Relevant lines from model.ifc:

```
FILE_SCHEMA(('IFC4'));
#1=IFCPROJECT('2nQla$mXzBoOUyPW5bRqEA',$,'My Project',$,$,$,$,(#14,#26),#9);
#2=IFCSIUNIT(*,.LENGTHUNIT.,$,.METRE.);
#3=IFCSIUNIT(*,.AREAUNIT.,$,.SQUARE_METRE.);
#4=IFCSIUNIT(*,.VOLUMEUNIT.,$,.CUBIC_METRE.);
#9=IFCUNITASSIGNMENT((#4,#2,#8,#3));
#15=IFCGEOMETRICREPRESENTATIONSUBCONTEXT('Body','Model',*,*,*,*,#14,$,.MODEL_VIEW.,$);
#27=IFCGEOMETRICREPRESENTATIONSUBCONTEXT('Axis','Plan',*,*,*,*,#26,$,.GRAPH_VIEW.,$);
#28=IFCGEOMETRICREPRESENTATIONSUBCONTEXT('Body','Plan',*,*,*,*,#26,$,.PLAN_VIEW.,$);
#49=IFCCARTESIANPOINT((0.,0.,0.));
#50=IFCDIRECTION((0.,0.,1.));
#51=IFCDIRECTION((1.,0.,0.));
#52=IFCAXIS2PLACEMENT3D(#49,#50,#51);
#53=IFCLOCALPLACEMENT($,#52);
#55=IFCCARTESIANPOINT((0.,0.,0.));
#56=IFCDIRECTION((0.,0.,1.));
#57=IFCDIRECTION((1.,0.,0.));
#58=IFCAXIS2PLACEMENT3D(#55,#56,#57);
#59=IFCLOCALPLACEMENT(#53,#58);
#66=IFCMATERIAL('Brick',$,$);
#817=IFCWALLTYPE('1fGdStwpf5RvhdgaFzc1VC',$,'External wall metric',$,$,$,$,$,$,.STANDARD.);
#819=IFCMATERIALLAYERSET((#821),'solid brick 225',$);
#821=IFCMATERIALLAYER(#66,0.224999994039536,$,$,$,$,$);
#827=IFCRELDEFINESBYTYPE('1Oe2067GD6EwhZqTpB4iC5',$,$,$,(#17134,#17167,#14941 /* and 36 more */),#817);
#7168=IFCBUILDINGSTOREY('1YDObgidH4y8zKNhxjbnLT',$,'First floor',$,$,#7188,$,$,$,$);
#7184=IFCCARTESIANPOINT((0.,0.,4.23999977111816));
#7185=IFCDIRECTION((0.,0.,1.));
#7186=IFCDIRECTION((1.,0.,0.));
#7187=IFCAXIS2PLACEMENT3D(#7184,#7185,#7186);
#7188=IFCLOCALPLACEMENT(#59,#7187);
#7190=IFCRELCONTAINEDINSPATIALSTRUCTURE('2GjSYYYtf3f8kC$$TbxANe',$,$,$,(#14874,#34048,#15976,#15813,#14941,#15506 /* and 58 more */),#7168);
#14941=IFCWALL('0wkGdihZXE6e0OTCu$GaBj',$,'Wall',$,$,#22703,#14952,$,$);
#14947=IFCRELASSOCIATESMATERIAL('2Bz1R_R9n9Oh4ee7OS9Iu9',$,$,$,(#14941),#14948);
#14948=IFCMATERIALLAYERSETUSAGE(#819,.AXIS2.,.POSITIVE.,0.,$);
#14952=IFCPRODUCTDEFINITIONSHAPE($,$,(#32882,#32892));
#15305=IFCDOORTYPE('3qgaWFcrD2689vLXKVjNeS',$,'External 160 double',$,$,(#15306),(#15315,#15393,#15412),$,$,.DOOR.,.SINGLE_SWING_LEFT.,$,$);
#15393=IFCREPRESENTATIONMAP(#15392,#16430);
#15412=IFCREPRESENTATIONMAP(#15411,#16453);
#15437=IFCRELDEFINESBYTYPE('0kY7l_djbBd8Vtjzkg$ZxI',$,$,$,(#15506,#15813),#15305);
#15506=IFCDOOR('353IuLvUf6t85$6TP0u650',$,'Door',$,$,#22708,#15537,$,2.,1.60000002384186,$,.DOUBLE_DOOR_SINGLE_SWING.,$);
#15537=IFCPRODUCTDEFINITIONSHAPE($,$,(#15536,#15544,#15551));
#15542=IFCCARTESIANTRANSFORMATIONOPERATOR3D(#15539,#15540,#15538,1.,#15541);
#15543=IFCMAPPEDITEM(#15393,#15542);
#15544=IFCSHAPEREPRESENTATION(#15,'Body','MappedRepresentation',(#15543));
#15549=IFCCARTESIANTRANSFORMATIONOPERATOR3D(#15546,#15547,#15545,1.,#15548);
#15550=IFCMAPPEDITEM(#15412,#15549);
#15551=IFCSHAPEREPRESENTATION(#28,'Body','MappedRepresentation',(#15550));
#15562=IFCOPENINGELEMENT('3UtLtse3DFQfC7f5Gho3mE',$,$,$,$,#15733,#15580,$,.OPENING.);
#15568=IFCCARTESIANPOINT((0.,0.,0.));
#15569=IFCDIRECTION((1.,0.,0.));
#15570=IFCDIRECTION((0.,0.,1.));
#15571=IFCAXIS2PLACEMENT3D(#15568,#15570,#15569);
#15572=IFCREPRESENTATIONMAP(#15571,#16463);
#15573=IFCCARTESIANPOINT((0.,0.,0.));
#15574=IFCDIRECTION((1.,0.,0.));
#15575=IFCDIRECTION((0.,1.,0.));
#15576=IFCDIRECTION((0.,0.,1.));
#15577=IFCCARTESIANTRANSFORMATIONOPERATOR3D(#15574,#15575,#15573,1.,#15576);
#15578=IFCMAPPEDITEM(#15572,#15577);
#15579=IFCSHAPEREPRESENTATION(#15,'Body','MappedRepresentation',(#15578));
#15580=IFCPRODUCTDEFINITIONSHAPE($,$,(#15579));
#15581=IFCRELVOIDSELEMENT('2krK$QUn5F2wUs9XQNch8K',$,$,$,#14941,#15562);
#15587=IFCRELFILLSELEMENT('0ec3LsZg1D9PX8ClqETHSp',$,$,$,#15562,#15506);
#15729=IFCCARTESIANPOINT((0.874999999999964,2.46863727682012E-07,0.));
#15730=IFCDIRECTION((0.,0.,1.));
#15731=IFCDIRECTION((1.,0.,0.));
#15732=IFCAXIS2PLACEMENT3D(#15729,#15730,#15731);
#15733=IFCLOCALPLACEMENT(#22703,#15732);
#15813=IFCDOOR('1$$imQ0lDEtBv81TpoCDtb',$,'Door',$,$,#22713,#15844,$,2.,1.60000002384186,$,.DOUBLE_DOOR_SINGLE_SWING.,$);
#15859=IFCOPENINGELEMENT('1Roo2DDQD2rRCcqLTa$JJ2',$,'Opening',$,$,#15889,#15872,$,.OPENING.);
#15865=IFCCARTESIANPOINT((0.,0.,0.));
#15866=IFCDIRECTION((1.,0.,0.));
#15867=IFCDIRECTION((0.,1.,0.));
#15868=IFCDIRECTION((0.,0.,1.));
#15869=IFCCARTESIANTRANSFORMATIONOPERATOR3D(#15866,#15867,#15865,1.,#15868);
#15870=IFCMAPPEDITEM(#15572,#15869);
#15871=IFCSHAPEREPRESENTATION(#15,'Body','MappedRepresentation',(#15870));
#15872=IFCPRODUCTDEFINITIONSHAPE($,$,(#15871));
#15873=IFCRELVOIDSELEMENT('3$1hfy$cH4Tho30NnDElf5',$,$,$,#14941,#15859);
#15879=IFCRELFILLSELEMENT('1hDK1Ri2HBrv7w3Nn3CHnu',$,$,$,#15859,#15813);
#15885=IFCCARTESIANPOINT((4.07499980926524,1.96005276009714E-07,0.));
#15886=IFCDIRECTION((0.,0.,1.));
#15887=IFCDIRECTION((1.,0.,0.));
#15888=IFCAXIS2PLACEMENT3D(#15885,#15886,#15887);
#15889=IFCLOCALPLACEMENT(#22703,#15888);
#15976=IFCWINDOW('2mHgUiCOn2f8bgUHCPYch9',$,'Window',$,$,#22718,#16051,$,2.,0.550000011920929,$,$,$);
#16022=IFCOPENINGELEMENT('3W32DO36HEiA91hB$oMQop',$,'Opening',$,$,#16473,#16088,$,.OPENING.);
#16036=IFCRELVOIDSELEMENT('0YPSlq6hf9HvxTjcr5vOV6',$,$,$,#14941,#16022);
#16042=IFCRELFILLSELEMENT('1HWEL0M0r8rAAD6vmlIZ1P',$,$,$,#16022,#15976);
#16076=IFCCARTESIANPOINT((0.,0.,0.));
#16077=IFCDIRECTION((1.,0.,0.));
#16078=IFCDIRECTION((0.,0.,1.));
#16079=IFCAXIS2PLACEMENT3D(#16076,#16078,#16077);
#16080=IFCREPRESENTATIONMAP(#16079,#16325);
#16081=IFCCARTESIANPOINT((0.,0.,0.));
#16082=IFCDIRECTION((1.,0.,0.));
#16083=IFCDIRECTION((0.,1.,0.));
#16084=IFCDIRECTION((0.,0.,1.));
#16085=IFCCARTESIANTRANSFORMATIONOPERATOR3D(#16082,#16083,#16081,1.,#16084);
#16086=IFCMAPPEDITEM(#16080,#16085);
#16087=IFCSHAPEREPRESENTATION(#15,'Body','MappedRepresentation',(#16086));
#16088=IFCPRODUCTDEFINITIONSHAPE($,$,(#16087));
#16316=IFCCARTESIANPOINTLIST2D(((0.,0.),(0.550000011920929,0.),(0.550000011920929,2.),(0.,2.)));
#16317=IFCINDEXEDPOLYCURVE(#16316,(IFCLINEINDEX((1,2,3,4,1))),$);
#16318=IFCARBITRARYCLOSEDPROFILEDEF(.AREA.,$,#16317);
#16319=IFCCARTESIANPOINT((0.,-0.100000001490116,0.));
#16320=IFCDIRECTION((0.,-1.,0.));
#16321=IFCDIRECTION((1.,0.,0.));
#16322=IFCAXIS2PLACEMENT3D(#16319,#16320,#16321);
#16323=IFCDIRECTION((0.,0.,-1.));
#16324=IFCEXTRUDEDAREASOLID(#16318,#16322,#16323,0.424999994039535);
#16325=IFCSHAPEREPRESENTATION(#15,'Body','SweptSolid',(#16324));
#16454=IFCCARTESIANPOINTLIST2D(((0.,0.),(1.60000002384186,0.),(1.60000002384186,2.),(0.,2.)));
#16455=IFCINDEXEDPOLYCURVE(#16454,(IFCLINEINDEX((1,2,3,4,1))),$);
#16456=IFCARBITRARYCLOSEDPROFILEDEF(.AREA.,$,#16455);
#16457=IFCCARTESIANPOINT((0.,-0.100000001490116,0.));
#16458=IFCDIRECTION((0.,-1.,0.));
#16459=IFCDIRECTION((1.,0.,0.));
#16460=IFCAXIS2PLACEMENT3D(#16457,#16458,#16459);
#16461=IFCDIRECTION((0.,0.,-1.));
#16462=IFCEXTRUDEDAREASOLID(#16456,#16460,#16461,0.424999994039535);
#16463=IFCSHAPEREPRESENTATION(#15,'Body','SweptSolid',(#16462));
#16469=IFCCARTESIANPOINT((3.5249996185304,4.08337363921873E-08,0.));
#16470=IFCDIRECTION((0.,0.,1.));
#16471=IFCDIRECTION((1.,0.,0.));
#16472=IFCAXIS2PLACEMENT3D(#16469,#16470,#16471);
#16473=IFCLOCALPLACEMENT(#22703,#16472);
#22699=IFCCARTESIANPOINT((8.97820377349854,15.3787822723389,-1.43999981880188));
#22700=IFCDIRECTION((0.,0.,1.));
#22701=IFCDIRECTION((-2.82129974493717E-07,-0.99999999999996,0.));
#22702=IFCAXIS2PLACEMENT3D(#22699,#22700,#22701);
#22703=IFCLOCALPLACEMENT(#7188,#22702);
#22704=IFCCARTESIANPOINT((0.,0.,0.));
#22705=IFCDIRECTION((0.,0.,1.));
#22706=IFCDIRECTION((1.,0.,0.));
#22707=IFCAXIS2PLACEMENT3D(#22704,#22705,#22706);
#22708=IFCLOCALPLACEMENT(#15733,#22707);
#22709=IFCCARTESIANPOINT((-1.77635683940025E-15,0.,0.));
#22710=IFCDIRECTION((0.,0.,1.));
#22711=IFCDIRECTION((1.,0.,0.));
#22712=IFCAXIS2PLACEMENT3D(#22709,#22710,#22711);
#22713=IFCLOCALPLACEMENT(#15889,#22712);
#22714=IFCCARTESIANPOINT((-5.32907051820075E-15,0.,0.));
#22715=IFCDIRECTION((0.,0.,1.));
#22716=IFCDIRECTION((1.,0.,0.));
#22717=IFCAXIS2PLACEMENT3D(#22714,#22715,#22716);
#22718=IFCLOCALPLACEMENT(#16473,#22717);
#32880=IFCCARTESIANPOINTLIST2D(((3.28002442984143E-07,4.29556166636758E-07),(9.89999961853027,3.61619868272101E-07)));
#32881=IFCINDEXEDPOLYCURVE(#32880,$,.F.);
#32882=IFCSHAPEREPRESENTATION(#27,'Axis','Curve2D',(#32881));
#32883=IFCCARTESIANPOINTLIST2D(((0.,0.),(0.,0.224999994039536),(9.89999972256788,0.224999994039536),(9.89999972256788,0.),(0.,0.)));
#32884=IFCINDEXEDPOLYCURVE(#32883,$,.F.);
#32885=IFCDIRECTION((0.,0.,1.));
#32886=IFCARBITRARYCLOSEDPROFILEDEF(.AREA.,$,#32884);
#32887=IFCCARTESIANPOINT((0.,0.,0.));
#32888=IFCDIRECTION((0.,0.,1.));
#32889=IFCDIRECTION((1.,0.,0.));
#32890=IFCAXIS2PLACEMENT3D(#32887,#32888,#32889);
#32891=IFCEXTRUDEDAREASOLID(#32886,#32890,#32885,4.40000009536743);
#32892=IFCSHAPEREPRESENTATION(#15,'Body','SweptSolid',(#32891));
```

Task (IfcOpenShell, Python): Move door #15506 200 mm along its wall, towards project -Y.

```python
import ifcopenshell
import ifcopenshell.api.geometry
import ifcopenshell.util.placement
import ifcopenshell.util.unit

model = ifcopenshell.open("model.ifc")
unit_scale = ifcopenshell.util.unit.calculate_unit_scale(model)

door = model.by_guid("353IuLvUf6t85$6TP0u650")
opening = door.FillsVoids[0].RelatingOpeningElement
wall = opening.VoidsElements[0].RelatingBuildingElement

wall_matrix = ifcopenshell.util.placement.get_local_placement(wall.ObjectPlacement)
shift = wall_matrix[:3, 0] * 0.2 / unit_scale
before = ifcopenshell.util.placement.get_local_placement(door.ObjectPlacement)[:3, 3].copy()

# The door is placed relative to its opening, so it follows when the opening moves.
matrix = ifcopenshell.util.placement.get_local_placement(opening.ObjectPlacement)
matrix[:3, 3] += shift
ifcopenshell.api.geometry.edit_object_placement(
    model, product=opening, matrix=matrix, is_si=False, should_transform_children=True
)

after = ifcopenshell.util.placement.get_local_placement(door.ObjectPlacement)[:3, 3]
print("door moved by", (after - before).round(3) + 0.0)

model.write("model-out.ifc")
```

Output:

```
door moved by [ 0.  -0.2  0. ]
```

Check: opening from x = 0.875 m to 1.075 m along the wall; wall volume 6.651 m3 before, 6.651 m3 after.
